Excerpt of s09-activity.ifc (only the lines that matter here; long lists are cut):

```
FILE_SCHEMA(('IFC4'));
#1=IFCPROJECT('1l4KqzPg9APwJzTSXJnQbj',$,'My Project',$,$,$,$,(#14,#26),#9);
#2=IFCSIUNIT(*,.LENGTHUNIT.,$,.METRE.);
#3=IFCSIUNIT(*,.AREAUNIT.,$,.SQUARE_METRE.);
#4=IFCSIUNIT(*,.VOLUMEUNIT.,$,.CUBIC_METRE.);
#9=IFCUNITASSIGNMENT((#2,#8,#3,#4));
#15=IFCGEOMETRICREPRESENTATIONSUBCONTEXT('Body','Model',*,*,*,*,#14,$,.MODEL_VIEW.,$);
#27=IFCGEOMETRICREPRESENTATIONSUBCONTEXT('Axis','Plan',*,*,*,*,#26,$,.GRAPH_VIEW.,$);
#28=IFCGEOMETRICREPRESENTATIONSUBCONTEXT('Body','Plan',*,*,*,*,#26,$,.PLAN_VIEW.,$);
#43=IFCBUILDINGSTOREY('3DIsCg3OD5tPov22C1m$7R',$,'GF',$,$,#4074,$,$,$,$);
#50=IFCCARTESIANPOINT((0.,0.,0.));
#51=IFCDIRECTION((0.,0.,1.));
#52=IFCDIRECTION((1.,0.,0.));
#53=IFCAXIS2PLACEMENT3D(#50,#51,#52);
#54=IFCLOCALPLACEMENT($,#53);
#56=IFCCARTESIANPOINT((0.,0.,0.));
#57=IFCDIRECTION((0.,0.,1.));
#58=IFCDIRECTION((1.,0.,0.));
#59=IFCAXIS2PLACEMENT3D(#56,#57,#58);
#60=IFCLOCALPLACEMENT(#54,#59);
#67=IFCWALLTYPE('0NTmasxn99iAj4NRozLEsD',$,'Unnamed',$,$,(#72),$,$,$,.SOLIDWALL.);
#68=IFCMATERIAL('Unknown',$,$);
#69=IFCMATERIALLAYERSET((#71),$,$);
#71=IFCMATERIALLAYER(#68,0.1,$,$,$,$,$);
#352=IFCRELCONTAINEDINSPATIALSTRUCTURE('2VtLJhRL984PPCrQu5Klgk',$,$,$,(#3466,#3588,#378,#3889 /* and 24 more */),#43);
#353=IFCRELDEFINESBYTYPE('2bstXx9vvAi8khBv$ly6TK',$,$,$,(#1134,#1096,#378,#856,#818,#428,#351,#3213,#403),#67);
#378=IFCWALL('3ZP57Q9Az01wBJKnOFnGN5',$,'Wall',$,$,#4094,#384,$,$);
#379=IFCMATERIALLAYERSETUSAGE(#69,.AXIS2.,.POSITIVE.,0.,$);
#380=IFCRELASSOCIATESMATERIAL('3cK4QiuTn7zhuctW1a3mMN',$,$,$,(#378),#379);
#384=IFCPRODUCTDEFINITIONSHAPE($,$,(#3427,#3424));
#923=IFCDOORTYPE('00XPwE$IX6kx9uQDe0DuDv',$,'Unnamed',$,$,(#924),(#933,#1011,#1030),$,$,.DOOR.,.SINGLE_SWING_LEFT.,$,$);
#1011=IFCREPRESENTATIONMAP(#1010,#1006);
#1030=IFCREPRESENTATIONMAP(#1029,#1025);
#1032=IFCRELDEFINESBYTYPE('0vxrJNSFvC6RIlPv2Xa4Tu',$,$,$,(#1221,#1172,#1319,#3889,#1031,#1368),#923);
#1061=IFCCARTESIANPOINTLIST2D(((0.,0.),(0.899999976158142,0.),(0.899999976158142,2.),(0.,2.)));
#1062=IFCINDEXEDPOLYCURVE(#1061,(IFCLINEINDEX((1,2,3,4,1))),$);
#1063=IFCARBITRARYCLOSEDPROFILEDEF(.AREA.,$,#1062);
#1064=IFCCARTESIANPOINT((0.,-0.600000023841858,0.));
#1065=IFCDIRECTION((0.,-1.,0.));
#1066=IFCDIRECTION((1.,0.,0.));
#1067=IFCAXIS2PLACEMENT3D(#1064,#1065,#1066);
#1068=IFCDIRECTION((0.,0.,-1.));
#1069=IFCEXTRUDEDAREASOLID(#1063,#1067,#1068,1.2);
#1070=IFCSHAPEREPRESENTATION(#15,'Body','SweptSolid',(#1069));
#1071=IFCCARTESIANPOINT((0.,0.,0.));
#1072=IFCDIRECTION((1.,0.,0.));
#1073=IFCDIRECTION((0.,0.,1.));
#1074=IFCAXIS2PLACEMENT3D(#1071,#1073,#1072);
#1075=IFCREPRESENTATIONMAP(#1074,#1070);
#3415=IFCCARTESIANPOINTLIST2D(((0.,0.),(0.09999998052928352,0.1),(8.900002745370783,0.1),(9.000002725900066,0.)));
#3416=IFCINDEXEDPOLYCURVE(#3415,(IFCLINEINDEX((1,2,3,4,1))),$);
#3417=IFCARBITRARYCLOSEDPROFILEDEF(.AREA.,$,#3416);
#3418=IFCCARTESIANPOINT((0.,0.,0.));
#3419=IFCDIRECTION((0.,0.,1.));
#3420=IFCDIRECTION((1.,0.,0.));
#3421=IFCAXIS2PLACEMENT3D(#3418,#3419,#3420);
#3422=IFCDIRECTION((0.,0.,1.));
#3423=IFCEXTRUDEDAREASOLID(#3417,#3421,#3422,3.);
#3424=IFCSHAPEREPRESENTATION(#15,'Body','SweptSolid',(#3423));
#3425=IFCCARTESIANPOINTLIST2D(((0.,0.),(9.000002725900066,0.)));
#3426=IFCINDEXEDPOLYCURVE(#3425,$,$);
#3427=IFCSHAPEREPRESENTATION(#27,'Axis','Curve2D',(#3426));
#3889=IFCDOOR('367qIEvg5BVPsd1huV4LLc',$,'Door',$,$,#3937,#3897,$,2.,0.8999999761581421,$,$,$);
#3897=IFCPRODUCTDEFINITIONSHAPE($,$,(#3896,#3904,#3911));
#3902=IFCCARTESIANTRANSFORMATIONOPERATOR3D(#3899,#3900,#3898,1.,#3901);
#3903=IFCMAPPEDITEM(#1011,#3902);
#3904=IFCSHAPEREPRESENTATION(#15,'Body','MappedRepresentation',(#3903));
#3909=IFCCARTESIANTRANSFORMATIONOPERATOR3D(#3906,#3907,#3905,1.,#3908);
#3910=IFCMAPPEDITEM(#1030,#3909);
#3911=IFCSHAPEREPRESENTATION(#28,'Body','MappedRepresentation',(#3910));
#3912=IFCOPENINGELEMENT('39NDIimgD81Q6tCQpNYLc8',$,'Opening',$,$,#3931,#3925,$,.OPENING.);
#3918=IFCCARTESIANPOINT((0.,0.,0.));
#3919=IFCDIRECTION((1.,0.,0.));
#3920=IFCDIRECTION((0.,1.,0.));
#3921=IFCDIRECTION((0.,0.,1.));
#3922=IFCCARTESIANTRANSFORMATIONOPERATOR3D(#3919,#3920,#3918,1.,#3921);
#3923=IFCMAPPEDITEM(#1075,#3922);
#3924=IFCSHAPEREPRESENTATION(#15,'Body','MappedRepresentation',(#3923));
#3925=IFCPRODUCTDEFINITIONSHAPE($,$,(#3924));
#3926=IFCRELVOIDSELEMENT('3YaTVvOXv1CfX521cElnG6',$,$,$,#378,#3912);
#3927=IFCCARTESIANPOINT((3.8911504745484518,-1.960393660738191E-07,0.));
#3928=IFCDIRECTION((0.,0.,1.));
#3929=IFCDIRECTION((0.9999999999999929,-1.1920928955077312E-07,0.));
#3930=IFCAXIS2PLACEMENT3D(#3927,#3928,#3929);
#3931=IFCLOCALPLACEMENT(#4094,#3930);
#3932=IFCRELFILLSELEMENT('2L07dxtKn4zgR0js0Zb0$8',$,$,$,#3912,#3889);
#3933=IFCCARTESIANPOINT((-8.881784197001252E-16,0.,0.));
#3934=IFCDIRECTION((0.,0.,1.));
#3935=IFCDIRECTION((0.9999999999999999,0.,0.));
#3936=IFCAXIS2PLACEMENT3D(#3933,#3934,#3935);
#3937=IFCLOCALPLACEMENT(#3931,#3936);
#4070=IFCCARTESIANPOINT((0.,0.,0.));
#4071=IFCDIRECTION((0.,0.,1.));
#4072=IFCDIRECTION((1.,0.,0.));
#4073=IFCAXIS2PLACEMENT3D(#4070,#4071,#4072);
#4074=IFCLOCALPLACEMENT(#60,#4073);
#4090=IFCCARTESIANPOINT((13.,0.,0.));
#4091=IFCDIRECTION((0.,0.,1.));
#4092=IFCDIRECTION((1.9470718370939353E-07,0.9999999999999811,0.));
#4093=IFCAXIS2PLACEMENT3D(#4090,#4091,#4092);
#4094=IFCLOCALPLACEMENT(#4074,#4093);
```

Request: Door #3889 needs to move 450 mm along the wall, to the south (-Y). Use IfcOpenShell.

```python
import ifcopenshell
import ifcopenshell.api.geometry
import ifcopenshell.util.placement

model = ifcopenshell.open("s09-activity.ifc")

door = model.by_guid("367qIEvg5BVPsd1huV4LLc")
opening = door.FillsVoids[0].RelatingOpeningElement
wall = opening.VoidsElements[0].RelatingBuildingElement

wall_matrix = ifcopenshell.util.placement.get_local_placement(wall.ObjectPlacement)
shift = wall_matrix[:3, 0] * -0.45
before = ifcopenshell.util.placement.get_local_placement(door.ObjectPlacement)[:3, 3].copy()

# The door is placed relative to its opening, so it follows when the opening moves.
matrix = ifcopenshell.util.placement.get_local_placement(opening.ObjectPlacement)
matrix[:3, 3] += shift
ifcopenshell.api.geometry.edit_object_placement(
    model, product=opening, matrix=matrix, is_si=False, should_transform_children=True
)

after = ifcopenshell.util.placement.get_local_placement(door.ObjectPlacement)[:3, 3]
print("door moved by", (after - before).round(3) + 0.0)

model.write("s09-activity_edited.ifc")
```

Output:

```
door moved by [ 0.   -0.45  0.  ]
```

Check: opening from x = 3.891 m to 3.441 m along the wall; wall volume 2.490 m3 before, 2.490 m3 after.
